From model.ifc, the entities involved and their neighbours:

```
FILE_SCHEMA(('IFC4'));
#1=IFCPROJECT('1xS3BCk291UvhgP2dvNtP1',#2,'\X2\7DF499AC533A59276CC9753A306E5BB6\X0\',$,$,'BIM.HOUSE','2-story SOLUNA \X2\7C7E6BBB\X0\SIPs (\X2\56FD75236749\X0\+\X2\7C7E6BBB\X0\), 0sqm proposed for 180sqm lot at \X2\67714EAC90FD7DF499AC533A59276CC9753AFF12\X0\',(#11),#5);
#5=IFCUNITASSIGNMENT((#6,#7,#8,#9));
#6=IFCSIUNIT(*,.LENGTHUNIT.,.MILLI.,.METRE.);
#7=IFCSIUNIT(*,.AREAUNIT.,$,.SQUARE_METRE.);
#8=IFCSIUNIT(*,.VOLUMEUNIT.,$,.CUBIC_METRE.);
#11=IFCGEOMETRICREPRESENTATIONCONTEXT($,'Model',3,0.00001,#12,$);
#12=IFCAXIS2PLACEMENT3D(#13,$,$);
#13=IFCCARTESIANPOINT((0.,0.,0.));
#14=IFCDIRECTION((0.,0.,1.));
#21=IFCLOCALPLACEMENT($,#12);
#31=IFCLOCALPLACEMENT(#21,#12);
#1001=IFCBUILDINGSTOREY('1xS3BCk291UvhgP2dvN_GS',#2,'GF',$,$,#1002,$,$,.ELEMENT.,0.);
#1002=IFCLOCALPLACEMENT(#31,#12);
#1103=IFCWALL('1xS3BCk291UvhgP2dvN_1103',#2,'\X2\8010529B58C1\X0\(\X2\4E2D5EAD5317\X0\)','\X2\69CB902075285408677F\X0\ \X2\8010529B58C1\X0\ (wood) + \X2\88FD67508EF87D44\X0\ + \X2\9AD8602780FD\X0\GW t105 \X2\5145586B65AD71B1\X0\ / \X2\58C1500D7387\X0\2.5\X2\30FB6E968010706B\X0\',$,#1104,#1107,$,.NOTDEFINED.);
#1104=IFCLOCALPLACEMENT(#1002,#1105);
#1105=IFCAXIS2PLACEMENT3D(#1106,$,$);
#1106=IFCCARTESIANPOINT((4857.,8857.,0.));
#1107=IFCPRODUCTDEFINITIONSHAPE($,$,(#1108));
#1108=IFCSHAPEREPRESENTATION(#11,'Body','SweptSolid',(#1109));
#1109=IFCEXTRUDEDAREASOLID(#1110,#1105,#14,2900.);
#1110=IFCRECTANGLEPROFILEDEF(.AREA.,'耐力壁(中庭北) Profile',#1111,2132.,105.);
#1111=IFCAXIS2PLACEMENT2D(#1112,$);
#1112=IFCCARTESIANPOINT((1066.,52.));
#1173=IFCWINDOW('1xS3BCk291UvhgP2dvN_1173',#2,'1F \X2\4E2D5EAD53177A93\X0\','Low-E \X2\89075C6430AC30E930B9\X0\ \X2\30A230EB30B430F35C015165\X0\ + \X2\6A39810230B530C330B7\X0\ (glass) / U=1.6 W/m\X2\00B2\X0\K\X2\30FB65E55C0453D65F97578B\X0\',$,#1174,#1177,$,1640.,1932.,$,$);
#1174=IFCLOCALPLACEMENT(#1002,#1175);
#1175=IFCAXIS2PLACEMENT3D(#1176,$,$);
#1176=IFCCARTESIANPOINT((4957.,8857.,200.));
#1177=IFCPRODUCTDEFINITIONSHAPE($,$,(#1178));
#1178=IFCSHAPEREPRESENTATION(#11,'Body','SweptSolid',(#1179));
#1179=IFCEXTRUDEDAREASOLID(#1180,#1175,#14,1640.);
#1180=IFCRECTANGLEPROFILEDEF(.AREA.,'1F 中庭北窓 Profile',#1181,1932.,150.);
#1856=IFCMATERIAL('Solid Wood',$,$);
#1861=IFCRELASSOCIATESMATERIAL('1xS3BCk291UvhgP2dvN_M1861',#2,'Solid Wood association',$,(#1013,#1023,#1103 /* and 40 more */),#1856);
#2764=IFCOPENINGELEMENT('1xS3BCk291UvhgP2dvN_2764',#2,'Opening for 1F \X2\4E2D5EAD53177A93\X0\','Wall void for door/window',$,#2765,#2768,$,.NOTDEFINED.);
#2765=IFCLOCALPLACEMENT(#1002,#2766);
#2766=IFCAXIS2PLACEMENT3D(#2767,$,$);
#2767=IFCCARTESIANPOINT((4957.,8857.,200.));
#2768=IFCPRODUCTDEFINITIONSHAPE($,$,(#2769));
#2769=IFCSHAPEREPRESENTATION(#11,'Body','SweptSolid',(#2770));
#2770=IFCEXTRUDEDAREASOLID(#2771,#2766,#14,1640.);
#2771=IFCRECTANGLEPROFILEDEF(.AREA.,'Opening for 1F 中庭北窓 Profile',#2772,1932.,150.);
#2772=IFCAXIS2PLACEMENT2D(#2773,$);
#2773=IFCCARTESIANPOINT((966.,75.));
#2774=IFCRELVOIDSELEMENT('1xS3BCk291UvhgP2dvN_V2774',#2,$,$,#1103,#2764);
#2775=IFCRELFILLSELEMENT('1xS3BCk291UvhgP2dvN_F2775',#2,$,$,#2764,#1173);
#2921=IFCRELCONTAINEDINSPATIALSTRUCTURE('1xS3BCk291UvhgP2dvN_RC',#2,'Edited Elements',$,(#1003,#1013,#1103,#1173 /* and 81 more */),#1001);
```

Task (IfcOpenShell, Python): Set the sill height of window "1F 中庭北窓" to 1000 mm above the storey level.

```python
import numpy as np
import ifcopenshell
import ifcopenshell.api.geometry
import ifcopenshell.geom
import ifcopenshell.util.element
import ifcopenshell.util.placement
import ifcopenshell.util.shape
import ifcopenshell.util.unit

model = ifcopenshell.open("model.ifc")
unit_scale = ifcopenshell.util.unit.calculate_unit_scale(model)

window = model.by_guid("1xS3BCk291UvhgP2dvN_1173")
opening = window.FillsVoids[0].RelatingOpeningElement
storey = ifcopenshell.util.element.get_container(window, ifc_class="IfcBuildingStorey")
level = ifcopenshell.util.placement.get_local_placement(storey.ObjectPlacement)[2, 3]

# The opening's origin need not be at the sill, so measure its lowest point.
shape = ifcopenshell.geom.create_shape(ifcopenshell.geom.settings(), opening)
bottom = ifcopenshell.util.shape.get_shape_bottom_elevation(shape, shape.geometry) / unit_scale
dz = level + 1 / unit_scale - bottom

shift = np.array([0.0, 0.0, dz])
# The window is not placed relative to its opening, so move both.
for product in (opening, window):
    matrix = ifcopenshell.util.placement.get_local_placement(product.ObjectPlacement)
    matrix[:3, 3] += shift
    ifcopenshell.api.geometry.edit_object_placement(model, product=product, matrix=matrix, is_si=False)

print(f"moved by {dz * unit_scale:+.3f} m")

model.write("model_v2.ifc")
```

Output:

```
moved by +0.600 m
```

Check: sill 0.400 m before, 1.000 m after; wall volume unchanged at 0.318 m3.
